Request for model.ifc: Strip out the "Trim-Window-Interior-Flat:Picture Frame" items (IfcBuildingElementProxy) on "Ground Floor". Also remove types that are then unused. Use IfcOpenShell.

First a look at what the model holds.

```python
import ifcopenshell
import ifcopenshell.util.element

model = ifcopenshell.open("model.ifc")
print(model.schema)
storey = next(s for s in model.by_type("IfcBuildingStorey") if s.Name == "Ground Floor")
proxies = [e for e in ifcopenshell.util.element.get_decomposition(storey) if e.is_a("IfcBuildingElementProxy")]
seen = {}
for e in proxies:
    element_type = ifcopenshell.util.element.get_type(e)
    name = element_type.Name if element_type not in (None, e) else None
    seen[name] = seen.get(name, 0) + 1
for name, count in sorted(seen.items(), key=str):
    print(count, "x", name)
```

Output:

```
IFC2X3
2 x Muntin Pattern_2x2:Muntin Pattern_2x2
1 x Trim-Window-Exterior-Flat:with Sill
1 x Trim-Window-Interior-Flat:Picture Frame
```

```python
import ifcopenshell
import ifcopenshell.api.root
import ifcopenshell.util.element

model = ifcopenshell.open("model.ifc")

storey = next(s for s in model.by_type("IfcBuildingStorey") if s.Name == "Ground Floor")
proxies = [e for e in ifcopenshell.util.element.get_decomposition(storey) if e.is_a("IfcBuildingElementProxy")]
targets = [e for e in proxies if (t := ifcopenshell.util.element.get_type(e)) not in (None, e) and t.Name == "Trim-Window-Interior-Flat:Picture Frame"]
types = {ifcopenshell.util.element.get_type(e) for e in targets} - {None, *targets}

for e in targets:
    ifcopenshell.api.root.remove_product(model, product=e)
print(len(targets), "removed")

unused = [t for t in types if not ifcopenshell.util.element.get_types(t)]
for t in unused:
    ifcopenshell.api.root.remove_product(model, product=t)
print(len(unused), "unused types removed")

model.write("model_updated.ifc")
```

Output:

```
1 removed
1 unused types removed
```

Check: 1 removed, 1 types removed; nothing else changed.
